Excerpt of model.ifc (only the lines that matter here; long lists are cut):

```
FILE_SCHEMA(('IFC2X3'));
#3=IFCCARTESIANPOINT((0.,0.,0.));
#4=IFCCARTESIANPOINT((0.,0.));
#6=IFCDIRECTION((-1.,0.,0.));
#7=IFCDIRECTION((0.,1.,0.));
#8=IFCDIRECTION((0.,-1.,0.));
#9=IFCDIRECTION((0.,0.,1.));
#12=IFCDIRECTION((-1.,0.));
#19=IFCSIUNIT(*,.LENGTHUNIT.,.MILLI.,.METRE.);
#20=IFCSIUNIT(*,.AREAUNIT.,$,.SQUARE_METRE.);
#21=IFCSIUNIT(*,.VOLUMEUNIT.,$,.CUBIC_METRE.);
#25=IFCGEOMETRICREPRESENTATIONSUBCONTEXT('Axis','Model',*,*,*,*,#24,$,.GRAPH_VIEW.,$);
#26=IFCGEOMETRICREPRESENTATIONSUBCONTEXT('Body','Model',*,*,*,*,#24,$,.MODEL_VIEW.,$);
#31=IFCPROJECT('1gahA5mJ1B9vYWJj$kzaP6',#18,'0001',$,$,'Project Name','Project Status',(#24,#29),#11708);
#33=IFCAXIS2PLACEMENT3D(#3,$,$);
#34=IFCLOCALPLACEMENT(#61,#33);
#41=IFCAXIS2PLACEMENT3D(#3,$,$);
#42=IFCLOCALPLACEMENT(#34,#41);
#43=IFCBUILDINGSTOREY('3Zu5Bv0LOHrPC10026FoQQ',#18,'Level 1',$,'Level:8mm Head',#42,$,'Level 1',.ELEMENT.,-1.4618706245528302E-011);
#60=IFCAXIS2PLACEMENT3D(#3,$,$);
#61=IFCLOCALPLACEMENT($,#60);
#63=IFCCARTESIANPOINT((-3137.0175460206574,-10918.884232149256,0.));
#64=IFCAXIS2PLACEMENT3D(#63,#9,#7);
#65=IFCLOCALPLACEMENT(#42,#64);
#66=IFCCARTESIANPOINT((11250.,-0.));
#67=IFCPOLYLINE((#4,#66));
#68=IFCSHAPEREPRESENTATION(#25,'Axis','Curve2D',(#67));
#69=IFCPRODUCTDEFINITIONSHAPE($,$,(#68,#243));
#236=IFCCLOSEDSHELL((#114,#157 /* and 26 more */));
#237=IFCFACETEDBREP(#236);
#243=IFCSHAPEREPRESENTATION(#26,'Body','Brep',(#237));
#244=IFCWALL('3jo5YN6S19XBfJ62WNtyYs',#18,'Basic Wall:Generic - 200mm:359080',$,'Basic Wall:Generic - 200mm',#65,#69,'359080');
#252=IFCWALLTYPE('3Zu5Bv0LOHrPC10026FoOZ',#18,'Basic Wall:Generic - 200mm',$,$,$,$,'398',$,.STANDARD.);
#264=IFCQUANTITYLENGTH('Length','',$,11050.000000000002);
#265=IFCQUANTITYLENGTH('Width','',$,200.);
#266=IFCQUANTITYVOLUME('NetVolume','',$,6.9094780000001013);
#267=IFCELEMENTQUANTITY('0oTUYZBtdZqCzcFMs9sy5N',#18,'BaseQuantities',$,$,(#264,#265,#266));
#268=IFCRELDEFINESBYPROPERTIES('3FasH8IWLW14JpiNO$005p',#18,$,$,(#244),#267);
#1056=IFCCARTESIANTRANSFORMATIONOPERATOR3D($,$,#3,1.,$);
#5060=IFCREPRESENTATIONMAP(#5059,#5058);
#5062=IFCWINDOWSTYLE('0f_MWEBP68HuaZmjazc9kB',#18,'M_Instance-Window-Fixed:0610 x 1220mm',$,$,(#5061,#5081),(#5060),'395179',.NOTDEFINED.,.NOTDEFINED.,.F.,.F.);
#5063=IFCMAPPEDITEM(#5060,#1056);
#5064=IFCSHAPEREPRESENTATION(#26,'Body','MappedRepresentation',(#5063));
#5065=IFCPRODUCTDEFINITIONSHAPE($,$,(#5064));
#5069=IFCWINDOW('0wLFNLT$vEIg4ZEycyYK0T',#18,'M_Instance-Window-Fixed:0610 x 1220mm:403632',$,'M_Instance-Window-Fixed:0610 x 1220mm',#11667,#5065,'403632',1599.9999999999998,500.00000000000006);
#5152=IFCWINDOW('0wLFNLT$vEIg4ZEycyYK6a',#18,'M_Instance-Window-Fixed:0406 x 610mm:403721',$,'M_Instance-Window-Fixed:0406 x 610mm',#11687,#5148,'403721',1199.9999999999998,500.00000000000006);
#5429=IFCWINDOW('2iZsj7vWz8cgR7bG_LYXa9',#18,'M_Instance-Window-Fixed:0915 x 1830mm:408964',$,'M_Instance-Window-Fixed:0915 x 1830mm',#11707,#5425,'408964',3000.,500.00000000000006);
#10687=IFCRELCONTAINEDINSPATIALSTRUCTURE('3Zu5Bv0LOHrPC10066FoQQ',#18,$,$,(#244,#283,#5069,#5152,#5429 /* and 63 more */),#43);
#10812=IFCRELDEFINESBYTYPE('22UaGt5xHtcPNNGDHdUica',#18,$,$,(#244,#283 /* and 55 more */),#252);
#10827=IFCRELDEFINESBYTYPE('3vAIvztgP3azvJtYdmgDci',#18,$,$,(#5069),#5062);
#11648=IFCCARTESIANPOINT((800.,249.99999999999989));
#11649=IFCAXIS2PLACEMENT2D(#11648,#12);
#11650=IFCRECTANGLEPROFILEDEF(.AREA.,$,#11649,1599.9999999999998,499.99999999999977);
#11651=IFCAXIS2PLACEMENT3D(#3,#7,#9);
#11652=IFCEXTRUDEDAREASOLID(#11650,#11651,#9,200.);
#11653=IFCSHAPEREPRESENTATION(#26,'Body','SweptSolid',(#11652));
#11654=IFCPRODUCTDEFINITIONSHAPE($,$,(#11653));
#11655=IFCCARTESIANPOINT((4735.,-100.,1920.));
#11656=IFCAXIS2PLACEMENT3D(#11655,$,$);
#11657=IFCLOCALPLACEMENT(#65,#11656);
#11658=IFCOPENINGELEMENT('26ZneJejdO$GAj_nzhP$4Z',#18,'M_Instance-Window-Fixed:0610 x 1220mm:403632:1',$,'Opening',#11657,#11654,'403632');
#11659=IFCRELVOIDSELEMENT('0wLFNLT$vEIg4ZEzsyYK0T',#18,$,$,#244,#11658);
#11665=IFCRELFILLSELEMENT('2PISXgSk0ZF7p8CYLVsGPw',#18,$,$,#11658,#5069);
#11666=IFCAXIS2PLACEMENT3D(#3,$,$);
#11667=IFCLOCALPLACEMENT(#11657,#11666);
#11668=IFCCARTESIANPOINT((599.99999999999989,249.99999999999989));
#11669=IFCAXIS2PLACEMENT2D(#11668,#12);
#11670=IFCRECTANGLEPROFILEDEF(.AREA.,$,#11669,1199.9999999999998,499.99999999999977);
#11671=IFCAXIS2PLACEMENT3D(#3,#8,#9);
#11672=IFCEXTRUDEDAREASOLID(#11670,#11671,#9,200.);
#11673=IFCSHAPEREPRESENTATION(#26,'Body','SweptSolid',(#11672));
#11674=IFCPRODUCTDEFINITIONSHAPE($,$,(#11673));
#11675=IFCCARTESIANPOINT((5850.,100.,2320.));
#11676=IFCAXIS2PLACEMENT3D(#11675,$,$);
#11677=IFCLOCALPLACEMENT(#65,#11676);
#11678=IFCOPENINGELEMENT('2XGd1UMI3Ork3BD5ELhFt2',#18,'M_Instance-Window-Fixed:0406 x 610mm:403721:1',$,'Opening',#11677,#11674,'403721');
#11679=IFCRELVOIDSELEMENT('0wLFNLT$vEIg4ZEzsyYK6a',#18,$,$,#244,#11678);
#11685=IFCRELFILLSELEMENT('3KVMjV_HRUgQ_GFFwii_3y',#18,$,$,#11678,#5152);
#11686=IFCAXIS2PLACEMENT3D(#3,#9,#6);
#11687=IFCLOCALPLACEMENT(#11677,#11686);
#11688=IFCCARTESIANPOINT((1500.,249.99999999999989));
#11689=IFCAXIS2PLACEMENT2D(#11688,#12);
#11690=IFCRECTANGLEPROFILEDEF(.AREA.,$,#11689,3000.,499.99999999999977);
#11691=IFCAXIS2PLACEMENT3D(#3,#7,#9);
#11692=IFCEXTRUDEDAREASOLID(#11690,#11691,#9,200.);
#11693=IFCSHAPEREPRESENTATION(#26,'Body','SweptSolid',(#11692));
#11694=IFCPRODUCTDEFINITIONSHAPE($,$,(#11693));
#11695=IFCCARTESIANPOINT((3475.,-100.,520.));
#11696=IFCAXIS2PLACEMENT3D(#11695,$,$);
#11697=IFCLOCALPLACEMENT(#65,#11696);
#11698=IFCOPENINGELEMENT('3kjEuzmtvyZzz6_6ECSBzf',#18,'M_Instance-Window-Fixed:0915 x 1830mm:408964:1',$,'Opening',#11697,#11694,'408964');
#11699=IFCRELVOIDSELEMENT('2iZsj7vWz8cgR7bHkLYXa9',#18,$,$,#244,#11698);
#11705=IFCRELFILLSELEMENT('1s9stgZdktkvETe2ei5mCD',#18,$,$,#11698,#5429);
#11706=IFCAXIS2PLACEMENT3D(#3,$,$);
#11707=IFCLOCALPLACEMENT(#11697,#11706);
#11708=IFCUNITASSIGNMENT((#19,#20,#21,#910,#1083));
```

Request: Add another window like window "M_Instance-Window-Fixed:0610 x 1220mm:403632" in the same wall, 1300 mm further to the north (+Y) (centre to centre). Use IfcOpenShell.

```python
import ifcopenshell
import ifcopenshell.api.feature
import ifcopenshell.api.geometry
import ifcopenshell.api.pset
import ifcopenshell.api.root
import ifcopenshell.geom
import ifcopenshell.util.element
import ifcopenshell.util.placement
import ifcopenshell.util.shape
import ifcopenshell.util.unit

model = ifcopenshell.open("model.ifc")
unit_scale = ifcopenshell.util.unit.calculate_unit_scale(model)
volume_scale = ifcopenshell.util.unit.calculate_unit_scale(model, "VOLUMEUNIT")
settings = ifcopenshell.geom.settings()


def volume(element):
    """Net volume in cubic metres, openings subtracted."""
    shape = ifcopenshell.geom.create_shape(settings, element)
    return ifcopenshell.util.shape.get_volume(shape.geometry)


def reuse_history(source, copy):
    """copy_class also copies each property set's owner history, people and application; keep the originals."""
    for rel in copy.IsDefinedBy:
        if rel.is_a("IfcRelDefinesByProperties") and (history := rel.RelatingPropertyDefinition.OwnerHistory):
            rel.RelatingPropertyDefinition.OwnerHistory = source.OwnerHistory
            ifcopenshell.util.element.remove_deep2(model, history)


window = model.by_guid("0wLFNLT$vEIg4ZEycyYK0T")
opening = window.FillsVoids[0].RelatingOpeningElement
wall = opening.VoidsElements[0].RelatingBuildingElement
before = volume(wall)
shift = ifcopenshell.util.placement.get_local_placement(wall.ObjectPlacement)[:3, 0] * 1.3 / unit_scale

# copy_class copies the void relationship, type, container and properties, but no geometry.
new_opening = ifcopenshell.api.root.copy_class(model, product=opening)
new_opening.Representation = ifcopenshell.util.element.copy_deep(
    model, opening.Representation, exclude=["IfcGeometricRepresentationContext", "IfcRepresentationMap"]
)
new_opening.Name = "M_Instance-Window-Fixed:0610 x 1220mm"
new_opening.Tag = None
reuse_history(opening, new_opening)
new_window = ifcopenshell.api.root.copy_class(model, product=window)
new_window.Representation = ifcopenshell.util.element.copy_deep(
    model, window.Representation, exclude=["IfcGeometricRepresentationContext", "IfcRepresentationMap"]
)
new_window.Name = "M_Instance-Window-Fixed:0610 x 1220mm"
new_window.Tag = None
reuse_history(window, new_window)
fills = ifcopenshell.api.feature.add_filling(model, opening=new_opening, element=new_window)
fills.OwnerHistory = new_window.OwnerHistory  # required in IFC2X3

for old, new in ((opening, new_opening), (window, new_window)):
    matrix = ifcopenshell.util.placement.get_local_placement(old.ObjectPlacement)
    matrix[:3, 3] += shift
    ifcopenshell.api.geometry.edit_object_placement(model, product=new, matrix=matrix, is_si=False)

after = volume(wall)

# Update the wall's stored quantities.
qto = model.by_id(ifcopenshell.util.element.get_pset(wall, "BaseQuantities", should_inherit=False)["id"])
ifcopenshell.api.pset.edit_qto(model, qto=qto, properties={"NetVolume": after / volume_scale})

print(f"wall volume {before:.3f} -> {after:.3f} m3")

model.write("model_rev.ifc")
```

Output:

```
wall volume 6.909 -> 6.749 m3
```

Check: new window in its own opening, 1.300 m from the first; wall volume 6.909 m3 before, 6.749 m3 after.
